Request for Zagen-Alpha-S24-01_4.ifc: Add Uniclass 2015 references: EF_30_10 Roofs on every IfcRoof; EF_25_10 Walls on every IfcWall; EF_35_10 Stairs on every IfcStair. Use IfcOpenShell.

First a look at what the model holds.

```python
import ifcopenshell

model = ifcopenshell.open("Zagen-Alpha-S24-01_4.ifc")
print(model.schema)
print("classifications:", [c.Name for c in model.by_type("IfcClassification")])
for ifc_class in ("IfcDoor", "IfcRoof", "IfcStair", "IfcWall", "IfcWindow"):
    print(ifc_class, len(model.by_type(ifc_class)))
```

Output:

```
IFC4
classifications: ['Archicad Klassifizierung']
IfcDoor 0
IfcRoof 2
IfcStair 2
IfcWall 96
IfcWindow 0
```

```python
import ifcopenshell
import ifcopenshell.api.classification

model = ifcopenshell.open("Zagen-Alpha-S24-01_4.ifc")

system = ifcopenshell.api.classification.add_classification(model, classification="Uniclass 2015")

codes = {
    "IfcRoof": ("EF_30_10", "Roofs"),
    "IfcWall": ("EF_25_10", "Walls"),
    "IfcStair": ("EF_35_10", "Stairs"),
}
for ifc_class, (code, name) in codes.items():
    products = model.by_type(ifc_class)
    ifcopenshell.api.classification.add_reference(
        model, products=products, classification=system, identification=code, name=name
    )
    print(code, len(products))

model.write("Zagen-Alpha-S24-01_4_v2.ifc")
```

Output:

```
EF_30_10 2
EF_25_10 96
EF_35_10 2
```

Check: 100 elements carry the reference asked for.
